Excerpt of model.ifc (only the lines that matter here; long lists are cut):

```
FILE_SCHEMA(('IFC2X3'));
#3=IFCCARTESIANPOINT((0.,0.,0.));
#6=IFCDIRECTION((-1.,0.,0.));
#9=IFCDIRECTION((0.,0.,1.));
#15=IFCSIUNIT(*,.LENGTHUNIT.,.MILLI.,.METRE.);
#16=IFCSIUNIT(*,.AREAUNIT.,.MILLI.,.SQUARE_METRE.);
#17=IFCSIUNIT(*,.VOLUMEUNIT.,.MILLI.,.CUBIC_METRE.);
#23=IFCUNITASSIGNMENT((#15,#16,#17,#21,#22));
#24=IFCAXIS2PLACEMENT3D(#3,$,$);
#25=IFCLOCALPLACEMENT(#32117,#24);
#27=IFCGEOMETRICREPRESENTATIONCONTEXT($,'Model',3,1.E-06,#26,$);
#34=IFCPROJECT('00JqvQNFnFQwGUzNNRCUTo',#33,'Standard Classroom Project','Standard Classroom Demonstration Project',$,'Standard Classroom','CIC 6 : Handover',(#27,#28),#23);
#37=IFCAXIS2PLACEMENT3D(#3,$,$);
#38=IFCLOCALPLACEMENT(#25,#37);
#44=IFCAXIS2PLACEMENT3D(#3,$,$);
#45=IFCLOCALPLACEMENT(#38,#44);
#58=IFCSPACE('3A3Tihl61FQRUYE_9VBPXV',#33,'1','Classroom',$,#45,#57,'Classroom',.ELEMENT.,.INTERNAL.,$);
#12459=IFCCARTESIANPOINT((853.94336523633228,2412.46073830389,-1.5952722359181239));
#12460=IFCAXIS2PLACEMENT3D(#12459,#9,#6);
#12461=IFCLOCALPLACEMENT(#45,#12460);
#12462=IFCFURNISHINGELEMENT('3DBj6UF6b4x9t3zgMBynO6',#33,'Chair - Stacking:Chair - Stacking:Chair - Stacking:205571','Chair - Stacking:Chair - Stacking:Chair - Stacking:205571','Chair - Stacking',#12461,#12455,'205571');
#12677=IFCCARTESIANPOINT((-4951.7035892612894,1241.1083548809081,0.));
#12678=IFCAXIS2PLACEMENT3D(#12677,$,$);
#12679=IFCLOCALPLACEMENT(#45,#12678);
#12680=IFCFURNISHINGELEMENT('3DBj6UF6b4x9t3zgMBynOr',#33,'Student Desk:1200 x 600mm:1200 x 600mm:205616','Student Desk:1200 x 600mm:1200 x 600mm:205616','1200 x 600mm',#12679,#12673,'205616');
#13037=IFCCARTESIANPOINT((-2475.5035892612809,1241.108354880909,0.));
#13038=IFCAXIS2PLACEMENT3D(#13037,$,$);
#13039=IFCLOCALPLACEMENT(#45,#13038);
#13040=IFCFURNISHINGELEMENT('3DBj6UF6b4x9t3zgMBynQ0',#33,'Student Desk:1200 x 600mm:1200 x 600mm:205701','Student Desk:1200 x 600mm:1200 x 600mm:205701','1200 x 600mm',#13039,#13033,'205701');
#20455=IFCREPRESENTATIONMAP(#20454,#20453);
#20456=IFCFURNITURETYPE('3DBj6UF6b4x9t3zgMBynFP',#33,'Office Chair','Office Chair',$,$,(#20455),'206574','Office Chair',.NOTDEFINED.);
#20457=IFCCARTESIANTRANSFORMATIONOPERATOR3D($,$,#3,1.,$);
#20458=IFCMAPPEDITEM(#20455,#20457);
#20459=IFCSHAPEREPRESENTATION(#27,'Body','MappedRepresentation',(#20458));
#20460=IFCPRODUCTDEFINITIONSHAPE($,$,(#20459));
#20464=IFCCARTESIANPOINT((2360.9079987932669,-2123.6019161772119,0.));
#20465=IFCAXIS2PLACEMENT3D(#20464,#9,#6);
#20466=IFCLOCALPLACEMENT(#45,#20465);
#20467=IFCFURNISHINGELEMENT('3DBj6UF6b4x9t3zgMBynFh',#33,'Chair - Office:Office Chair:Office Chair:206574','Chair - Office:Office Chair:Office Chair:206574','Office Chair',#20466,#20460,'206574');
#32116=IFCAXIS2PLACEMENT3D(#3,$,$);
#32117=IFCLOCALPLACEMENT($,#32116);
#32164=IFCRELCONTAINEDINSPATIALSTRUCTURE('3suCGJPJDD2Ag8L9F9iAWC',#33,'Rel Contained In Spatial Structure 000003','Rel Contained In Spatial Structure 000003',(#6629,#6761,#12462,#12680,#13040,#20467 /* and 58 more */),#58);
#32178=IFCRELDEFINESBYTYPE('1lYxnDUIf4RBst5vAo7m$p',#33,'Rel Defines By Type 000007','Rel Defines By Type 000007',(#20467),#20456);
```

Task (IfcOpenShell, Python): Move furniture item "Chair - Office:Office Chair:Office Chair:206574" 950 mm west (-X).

```python
import ifcopenshell
import ifcopenshell.api.geometry
import ifcopenshell.util.placement

model = ifcopenshell.open("model.ifc")

item = model.by_id(20467)
matrix = ifcopenshell.util.placement.get_local_placement(item.ObjectPlacement)
matrix[0, 3] -= 950.0
ifcopenshell.api.geometry.edit_object_placement(model, product=item, matrix=matrix, is_si=False)

print(ifcopenshell.util.placement.get_local_placement(item.ObjectPlacement).round(3) + 0.0)

model.write("model_rev.ifc")
```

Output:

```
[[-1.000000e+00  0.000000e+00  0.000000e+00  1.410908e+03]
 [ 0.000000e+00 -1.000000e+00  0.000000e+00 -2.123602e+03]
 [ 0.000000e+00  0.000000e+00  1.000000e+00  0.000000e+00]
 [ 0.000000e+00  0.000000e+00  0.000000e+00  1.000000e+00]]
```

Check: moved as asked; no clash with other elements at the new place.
